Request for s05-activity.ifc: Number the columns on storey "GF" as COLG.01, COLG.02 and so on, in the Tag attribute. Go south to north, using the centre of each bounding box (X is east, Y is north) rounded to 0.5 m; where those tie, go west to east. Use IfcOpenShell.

First a look at what the model holds.

```python
import ifcopenshell
import ifcopenshell.util.element
import ifcopenshell.util.placement

model = ifcopenshell.open("s05-activity.ifc")
print(model.schema)
storey = next(s for s in model.by_type("IfcBuildingStorey") if s.Name == "GF")
columns = [e for e in ifcopenshell.util.element.get_decomposition(storey) if e.is_a("IfcColumn")]
for e in sorted(columns, key=lambda e: e.id()):
    origin = ifcopenshell.util.placement.get_local_placement(e.ObjectPlacement)[:3, 3]
    print(e.id(), e.Tag, e.Name, origin.round(2) + 0.0, sep=" | ")
```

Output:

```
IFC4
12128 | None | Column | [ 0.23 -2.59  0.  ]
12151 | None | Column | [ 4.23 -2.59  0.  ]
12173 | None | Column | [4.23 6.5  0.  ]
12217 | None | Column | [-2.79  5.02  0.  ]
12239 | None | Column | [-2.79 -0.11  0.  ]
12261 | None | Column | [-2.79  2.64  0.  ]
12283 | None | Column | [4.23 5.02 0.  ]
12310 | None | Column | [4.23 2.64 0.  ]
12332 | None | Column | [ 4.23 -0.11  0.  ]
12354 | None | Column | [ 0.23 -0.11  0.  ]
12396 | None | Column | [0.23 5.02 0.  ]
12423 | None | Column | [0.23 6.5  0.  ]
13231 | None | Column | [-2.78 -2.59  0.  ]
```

```python
import ifcopenshell
import ifcopenshell.geom
import ifcopenshell.util.element
import ifcopenshell.util.shape

model = ifcopenshell.open("s05-activity.ifc")
settings = ifcopenshell.geom.settings()
settings.set("use-world-coords", True)


def centre(element):
    shape = ifcopenshell.geom.create_shape(settings, element)
    return ifcopenshell.util.shape.get_bbox_centroid(shape.geometry)


storey = next(s for s in model.by_type("IfcBuildingStorey") if s.Name == "GF")
columns = [e for e in ifcopenshell.util.element.get_decomposition(storey) if e.is_a("IfcColumn")]

# Insertion points can sit at a corner or the storey origin, so sort by the geometry (in metres).
centres = {e: centre(e) for e in columns}
columns.sort(key=lambda e: (round(centres[e][1] / 0.5), centres[e][0]))

for i, e in enumerate(columns, start=1):
    number = f"COLG.{i:02d}"
    e.Tag = number
    print(e.id(), number)

model.write("s05-activity_updated.ifc")
```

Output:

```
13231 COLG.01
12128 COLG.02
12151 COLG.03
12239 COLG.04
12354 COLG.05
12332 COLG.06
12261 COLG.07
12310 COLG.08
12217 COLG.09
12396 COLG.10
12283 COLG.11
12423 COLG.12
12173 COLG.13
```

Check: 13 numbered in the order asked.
